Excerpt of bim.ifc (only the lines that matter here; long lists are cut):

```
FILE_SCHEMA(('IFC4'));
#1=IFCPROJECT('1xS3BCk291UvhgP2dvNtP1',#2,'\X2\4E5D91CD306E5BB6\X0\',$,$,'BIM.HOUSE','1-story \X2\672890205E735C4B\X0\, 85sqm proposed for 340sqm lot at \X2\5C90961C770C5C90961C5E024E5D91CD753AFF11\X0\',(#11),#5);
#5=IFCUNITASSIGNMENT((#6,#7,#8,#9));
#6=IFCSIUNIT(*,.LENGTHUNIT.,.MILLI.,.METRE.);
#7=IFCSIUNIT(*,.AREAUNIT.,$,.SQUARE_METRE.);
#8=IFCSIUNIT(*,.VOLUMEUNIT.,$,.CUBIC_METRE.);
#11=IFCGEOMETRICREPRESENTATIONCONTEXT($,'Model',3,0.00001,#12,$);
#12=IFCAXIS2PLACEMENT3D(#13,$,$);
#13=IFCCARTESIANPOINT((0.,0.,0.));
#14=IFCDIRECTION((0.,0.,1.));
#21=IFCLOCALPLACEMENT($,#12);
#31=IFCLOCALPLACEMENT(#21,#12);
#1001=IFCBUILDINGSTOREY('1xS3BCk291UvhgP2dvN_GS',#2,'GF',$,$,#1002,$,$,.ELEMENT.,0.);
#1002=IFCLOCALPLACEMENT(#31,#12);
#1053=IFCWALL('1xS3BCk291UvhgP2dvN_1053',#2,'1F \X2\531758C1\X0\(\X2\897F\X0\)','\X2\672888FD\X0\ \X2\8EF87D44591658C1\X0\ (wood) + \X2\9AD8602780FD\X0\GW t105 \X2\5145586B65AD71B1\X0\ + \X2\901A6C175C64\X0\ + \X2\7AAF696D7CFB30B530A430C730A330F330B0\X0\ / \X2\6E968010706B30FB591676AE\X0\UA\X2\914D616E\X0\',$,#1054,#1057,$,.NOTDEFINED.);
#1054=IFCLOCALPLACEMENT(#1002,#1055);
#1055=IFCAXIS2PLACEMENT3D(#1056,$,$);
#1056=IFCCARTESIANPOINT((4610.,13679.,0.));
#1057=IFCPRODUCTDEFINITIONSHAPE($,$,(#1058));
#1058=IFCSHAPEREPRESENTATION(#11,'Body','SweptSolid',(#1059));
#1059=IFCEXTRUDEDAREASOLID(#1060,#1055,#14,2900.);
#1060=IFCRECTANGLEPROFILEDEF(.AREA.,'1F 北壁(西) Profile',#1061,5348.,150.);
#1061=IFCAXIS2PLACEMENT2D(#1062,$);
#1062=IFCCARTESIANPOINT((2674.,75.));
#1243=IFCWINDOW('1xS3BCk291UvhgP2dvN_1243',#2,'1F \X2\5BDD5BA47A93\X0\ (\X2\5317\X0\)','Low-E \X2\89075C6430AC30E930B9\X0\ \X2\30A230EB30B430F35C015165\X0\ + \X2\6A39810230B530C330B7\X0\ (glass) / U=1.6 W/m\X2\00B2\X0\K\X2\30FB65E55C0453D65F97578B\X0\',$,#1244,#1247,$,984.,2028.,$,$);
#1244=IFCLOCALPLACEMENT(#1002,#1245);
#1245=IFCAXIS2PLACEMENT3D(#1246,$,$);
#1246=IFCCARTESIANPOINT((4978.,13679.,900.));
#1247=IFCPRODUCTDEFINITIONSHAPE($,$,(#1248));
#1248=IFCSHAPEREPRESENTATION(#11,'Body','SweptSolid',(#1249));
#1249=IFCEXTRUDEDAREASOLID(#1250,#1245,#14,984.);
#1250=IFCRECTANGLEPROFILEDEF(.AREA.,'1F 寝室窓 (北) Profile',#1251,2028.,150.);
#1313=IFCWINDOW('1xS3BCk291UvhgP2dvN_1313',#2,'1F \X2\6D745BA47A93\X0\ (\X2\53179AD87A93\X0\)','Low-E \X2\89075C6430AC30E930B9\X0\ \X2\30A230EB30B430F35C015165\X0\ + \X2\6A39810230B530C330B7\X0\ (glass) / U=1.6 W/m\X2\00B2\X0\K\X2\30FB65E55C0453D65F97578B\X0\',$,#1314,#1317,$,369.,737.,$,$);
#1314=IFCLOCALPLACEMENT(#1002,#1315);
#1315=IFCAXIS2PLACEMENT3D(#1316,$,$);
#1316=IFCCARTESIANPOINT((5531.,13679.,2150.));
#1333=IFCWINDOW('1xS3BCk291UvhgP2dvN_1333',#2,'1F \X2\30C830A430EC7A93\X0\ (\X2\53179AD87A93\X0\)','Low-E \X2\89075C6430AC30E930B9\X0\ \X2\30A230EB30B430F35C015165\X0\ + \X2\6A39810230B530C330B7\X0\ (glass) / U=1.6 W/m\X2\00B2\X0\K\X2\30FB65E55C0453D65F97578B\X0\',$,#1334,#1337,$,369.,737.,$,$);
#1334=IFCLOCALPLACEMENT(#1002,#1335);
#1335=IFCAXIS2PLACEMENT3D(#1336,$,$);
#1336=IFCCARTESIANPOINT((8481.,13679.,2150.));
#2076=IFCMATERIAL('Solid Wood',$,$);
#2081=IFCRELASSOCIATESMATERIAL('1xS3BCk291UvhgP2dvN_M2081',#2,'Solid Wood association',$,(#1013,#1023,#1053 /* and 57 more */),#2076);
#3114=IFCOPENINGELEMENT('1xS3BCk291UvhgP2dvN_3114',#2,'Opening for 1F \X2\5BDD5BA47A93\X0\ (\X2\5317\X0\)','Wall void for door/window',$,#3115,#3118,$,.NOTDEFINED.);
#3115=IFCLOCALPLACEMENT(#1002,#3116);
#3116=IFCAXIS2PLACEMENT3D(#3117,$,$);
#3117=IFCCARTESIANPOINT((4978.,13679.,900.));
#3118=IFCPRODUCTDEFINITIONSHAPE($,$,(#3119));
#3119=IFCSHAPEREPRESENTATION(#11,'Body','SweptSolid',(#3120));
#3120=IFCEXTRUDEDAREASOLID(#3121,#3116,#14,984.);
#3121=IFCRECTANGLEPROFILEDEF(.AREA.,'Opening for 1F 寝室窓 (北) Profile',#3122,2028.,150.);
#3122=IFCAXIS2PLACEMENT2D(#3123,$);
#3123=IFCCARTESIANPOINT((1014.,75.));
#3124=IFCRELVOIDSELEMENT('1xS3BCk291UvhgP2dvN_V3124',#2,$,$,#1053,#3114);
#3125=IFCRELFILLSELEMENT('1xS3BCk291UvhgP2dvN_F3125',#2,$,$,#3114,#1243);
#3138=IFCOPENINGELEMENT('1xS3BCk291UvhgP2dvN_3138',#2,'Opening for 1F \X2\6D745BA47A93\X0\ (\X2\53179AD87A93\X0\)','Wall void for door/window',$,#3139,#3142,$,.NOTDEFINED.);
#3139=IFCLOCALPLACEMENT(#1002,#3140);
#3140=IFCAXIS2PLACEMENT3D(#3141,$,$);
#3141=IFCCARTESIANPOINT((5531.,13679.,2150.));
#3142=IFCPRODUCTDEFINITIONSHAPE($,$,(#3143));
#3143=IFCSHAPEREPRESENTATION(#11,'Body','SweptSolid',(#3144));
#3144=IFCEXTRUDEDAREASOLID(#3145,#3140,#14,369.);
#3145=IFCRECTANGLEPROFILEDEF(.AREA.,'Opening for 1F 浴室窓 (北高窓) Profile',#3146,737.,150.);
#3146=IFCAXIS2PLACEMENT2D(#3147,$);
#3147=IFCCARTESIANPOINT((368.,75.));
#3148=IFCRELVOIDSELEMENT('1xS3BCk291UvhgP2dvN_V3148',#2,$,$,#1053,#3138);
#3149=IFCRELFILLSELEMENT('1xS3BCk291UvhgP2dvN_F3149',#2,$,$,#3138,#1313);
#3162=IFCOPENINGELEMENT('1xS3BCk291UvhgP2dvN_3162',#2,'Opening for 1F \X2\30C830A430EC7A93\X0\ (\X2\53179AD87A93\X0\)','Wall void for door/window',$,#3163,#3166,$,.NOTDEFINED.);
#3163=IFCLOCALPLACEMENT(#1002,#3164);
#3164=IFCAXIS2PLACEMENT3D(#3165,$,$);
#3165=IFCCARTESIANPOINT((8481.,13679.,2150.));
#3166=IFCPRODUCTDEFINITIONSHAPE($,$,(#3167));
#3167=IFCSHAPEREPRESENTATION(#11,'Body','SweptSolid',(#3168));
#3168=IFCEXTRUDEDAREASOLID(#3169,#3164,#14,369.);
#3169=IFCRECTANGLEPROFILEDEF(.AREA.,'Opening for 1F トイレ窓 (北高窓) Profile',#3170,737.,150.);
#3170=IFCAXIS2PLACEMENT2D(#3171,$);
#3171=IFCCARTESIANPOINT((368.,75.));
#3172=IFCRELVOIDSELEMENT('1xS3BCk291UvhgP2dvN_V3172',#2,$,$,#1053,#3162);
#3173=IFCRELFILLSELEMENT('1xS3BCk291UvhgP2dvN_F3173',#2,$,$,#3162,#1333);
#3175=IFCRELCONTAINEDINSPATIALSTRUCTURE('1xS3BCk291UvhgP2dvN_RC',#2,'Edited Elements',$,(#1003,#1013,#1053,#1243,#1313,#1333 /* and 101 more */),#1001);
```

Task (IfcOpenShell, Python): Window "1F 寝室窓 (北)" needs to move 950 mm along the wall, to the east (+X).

```python
import ifcopenshell
import ifcopenshell.api.geometry
import ifcopenshell.util.placement
import ifcopenshell.util.unit

model = ifcopenshell.open("bim.ifc")
unit_scale = ifcopenshell.util.unit.calculate_unit_scale(model)

window = model.by_guid("1xS3BCk291UvhgP2dvN_1243")
opening = window.FillsVoids[0].RelatingOpeningElement
wall = opening.VoidsElements[0].RelatingBuildingElement

wall_matrix = ifcopenshell.util.placement.get_local_placement(wall.ObjectPlacement)
shift = wall_matrix[:3, 0] * 0.95 / unit_scale
before = ifcopenshell.util.placement.get_local_placement(window.ObjectPlacement)[:3, 3].copy()

# The window is not placed relative to its opening, so move both.
for product in (opening, window):
    matrix = ifcopenshell.util.placement.get_local_placement(product.ObjectPlacement)
    matrix[:3, 3] += shift
    ifcopenshell.api.geometry.edit_object_placement(model, product=product, matrix=matrix, is_si=False)

after = ifcopenshell.util.placement.get_local_placement(window.ObjectPlacement)[:3, 3]
print("window moved by", (after - before).round(3) + 0.0)

model.write("bim_updated.ifc")
```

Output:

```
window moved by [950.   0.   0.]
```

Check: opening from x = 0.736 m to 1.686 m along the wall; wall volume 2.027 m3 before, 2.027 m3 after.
